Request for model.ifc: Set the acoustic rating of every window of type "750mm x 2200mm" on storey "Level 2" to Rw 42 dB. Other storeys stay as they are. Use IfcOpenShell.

First a look at what the model holds.

```python
import ifcopenshell
import ifcopenshell.util.element

model = ifcopenshell.open("model.ifc")
print(model.schema)
storey = next(s for s in model.by_type("IfcBuildingStorey") if s.Name == "Level 2")
windows = [e for e in ifcopenshell.util.element.get_decomposition(storey) if e.is_a("IfcWindow")]
seen = {}
for e in windows:
    element_type = ifcopenshell.util.element.get_type(e)
    key = (element_type.Name if element_type != e and element_type else None, ifcopenshell.util.element.get_pset(e, "Pset_WindowCommon", "AcousticRating"))
    seen[key] = seen.get(key, 0) + 1
for (name, value), count in sorted(seen.items(), key=str):
    print(count, "x", name, "|", value)
```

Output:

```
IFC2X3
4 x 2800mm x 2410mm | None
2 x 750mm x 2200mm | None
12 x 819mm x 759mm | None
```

```python
import ifcopenshell
import ifcopenshell.api.pset
import ifcopenshell.util.element

model = ifcopenshell.open("model.ifc")

storey = next(s for s in model.by_type("IfcBuildingStorey") if s.Name == "Level 2")
windows = [e for e in ifcopenshell.util.element.get_decomposition(storey) if e.is_a("IfcWindow")]

count = 0
for e in windows:
    element_type = ifcopenshell.util.element.get_type(e)
    if element_type in (None, e) or element_type.Name != "750mm x 2200mm":
        continue
    # add_pset returns the element's existing set when there is one.
    pset = ifcopenshell.api.pset.add_pset(model, product=e, name="Pset_WindowCommon")
    ifcopenshell.api.pset.edit_pset(model, pset=pset, properties={"AcousticRating": "Rw 42 dB"})
    count += 1

print(count, "windows updated")

model.write("model_edited.ifc")
```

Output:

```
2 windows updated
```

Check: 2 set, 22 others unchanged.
